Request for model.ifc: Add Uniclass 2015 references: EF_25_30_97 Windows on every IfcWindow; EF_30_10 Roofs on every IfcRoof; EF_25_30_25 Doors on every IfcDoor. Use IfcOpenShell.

First a look at what the model holds.

```python
import ifcopenshell

model = ifcopenshell.open("model.ifc")
print(model.schema)
print("classifications:", [c.Name for c in model.by_type("IfcClassification")])
for ifc_class in ("IfcDoor", "IfcRoof", "IfcStair", "IfcWall", "IfcWindow"):
    print(ifc_class, len(model.by_type(ifc_class)))
```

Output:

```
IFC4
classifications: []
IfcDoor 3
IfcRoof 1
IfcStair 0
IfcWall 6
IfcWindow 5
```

```python
import ifcopenshell
import ifcopenshell.api.classification

model = ifcopenshell.open("model.ifc")

system = ifcopenshell.api.classification.add_classification(model, classification="Uniclass 2015")

codes = {
    "IfcWindow": ("EF_25_30_97", "Windows"),
    "IfcRoof": ("EF_30_10", "Roofs"),
    "IfcDoor": ("EF_25_30_25", "Doors"),
}
for ifc_class, (code, name) in codes.items():
    products = model.by_type(ifc_class)
    ifcopenshell.api.classification.add_reference(
        model, products=products, classification=system, identification=code, name=name
    )
    print(code, len(products))

model.write("model_rev.ifc")
```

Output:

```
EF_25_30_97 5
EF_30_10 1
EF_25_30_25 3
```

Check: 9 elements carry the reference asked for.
